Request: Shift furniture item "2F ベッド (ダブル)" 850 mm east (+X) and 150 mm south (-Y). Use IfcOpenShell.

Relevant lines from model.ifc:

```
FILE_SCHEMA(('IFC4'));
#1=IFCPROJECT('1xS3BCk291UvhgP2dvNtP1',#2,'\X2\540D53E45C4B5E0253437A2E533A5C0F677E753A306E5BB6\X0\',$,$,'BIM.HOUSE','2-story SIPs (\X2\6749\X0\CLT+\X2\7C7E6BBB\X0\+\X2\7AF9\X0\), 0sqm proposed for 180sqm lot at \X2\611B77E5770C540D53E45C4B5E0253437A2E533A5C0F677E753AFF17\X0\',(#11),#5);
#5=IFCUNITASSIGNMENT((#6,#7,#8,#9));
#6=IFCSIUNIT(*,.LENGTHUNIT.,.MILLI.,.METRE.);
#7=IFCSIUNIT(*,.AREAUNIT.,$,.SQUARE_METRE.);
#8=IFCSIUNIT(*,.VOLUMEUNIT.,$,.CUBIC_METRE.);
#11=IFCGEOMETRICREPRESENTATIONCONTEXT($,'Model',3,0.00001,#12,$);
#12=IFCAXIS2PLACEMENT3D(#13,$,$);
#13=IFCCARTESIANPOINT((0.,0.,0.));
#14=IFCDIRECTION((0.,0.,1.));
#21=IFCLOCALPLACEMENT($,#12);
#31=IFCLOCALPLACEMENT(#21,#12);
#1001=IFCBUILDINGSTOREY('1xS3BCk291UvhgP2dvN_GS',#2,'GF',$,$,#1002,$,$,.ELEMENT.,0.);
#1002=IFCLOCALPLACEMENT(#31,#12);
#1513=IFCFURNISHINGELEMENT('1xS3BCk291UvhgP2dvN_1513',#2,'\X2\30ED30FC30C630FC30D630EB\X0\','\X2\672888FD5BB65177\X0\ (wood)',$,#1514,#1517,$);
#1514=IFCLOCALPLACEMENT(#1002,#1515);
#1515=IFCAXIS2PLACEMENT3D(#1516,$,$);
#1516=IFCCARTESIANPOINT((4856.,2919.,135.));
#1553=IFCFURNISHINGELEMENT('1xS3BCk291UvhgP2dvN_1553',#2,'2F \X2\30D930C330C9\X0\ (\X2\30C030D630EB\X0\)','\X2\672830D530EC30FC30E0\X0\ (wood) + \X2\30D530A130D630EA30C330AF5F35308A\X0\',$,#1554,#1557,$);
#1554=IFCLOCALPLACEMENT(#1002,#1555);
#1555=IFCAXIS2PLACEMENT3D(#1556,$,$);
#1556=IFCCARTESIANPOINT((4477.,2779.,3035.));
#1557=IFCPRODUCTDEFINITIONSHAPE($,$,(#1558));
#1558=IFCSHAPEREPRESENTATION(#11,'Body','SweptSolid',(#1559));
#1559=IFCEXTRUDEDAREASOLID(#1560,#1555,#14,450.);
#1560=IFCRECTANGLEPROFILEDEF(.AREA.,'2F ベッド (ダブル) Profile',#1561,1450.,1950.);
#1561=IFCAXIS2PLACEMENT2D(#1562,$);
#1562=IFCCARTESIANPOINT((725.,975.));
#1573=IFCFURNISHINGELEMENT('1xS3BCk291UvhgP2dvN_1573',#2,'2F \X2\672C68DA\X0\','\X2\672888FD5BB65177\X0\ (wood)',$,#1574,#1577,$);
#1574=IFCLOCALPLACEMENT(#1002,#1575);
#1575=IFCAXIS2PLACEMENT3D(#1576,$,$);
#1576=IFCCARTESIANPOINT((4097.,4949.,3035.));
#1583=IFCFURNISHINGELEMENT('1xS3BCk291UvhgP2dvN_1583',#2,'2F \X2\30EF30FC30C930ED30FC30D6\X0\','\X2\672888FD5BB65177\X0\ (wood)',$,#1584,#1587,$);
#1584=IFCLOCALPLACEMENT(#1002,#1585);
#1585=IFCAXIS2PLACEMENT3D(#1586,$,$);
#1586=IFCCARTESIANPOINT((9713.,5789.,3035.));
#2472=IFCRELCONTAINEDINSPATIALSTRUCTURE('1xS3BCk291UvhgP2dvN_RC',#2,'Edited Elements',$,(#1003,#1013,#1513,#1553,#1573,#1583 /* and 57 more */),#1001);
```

```python
import ifcopenshell
import ifcopenshell.api.geometry
import ifcopenshell.util.placement
import ifcopenshell.util.unit

model = ifcopenshell.open("model.ifc")
unit_scale = ifcopenshell.util.unit.calculate_unit_scale(model)

item = model.by_guid("1xS3BCk291UvhgP2dvN_1553")
matrix = ifcopenshell.util.placement.get_local_placement(item.ObjectPlacement)
matrix[0, 3] += 0.85 / unit_scale
matrix[1, 3] -= 0.15 / unit_scale
ifcopenshell.api.geometry.edit_object_placement(model, product=item, matrix=matrix, is_si=False)

print(ifcopenshell.util.placement.get_local_placement(item.ObjectPlacement).round(3) + 0.0)

model.write("model_rev.ifc")
```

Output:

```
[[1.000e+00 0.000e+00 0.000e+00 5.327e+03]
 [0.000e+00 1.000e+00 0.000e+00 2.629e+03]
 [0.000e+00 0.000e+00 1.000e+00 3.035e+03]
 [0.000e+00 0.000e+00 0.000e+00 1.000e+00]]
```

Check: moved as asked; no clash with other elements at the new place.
